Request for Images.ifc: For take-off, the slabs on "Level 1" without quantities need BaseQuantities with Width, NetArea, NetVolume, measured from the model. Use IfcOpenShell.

First a look at what the model holds.

```python
import ifcopenshell
import ifcopenshell.util.element
import ifcopenshell.util.unit

model = ifcopenshell.open("Images.ifc")
print(model.schema)
for unit_type in ("LENGTHUNIT", "AREAUNIT", "VOLUMEUNIT"):
    print(unit_type, ifcopenshell.util.unit.calculate_unit_scale(model, unit_type))
storey = next(s for s in model.by_type("IfcBuildingStorey") if s.Name == "Level 1")
slabs = [e for e in ifcopenshell.util.element.get_decomposition(storey) if e.is_a("IfcSlab")]
for e in sorted(slabs, key=lambda e: e.id()):
    print(e.id(), e.is_a(), e.Name, list(ifcopenshell.util.element.get_psets(e, qtos_only=True)), sep=" | ")
```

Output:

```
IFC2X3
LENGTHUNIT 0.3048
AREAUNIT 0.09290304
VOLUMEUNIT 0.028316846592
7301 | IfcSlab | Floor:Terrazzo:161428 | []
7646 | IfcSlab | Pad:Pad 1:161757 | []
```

```python
import ifcopenshell
import ifcopenshell.api.pset
import ifcopenshell.geom
import ifcopenshell.util.element
import ifcopenshell.util.shape
import ifcopenshell.util.unit

model = ifcopenshell.open("Images.ifc")
unit_scale = ifcopenshell.util.unit.calculate_unit_scale(model)
area_scale = ifcopenshell.util.unit.calculate_unit_scale(model, "AREAUNIT")
volume_scale = ifcopenshell.util.unit.calculate_unit_scale(model, "VOLUMEUNIT")
settings = ifcopenshell.geom.settings()

storey = next(s for s in model.by_type("IfcBuildingStorey") if s.Name == "Level 1")
slabs = [e for e in ifcopenshell.util.element.get_decomposition(storey) if e.is_a("IfcSlab")]

for e in sorted(slabs, key=lambda e: e.id()):
    if ifcopenshell.util.element.get_psets(e, qtos_only=True, should_inherit=False):
        continue
    # Geometry comes back in metres, in the element's own axes.
    shape = ifcopenshell.geom.create_shape(settings, e)
    values = {
        "Width": ifcopenshell.util.shape.get_z(shape.geometry) / unit_scale,
        "NetArea": ifcopenshell.util.shape.get_footprint_area(shape.geometry) / area_scale,
        "NetVolume": ifcopenshell.util.shape.get_volume(shape.geometry) / volume_scale,
    }
    qto = ifcopenshell.api.pset.add_qto(model, product=e, name="BaseQuantities")
    ifcopenshell.api.pset.edit_qto(model, qto=qto, properties=values)
    print(e.id(), {k: round(v, 3) for k, v in values.items()})

model.write("Images-out.ifc")
```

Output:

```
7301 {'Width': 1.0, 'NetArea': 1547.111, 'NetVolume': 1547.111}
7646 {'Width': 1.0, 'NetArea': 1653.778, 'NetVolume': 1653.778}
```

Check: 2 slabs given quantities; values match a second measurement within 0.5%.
